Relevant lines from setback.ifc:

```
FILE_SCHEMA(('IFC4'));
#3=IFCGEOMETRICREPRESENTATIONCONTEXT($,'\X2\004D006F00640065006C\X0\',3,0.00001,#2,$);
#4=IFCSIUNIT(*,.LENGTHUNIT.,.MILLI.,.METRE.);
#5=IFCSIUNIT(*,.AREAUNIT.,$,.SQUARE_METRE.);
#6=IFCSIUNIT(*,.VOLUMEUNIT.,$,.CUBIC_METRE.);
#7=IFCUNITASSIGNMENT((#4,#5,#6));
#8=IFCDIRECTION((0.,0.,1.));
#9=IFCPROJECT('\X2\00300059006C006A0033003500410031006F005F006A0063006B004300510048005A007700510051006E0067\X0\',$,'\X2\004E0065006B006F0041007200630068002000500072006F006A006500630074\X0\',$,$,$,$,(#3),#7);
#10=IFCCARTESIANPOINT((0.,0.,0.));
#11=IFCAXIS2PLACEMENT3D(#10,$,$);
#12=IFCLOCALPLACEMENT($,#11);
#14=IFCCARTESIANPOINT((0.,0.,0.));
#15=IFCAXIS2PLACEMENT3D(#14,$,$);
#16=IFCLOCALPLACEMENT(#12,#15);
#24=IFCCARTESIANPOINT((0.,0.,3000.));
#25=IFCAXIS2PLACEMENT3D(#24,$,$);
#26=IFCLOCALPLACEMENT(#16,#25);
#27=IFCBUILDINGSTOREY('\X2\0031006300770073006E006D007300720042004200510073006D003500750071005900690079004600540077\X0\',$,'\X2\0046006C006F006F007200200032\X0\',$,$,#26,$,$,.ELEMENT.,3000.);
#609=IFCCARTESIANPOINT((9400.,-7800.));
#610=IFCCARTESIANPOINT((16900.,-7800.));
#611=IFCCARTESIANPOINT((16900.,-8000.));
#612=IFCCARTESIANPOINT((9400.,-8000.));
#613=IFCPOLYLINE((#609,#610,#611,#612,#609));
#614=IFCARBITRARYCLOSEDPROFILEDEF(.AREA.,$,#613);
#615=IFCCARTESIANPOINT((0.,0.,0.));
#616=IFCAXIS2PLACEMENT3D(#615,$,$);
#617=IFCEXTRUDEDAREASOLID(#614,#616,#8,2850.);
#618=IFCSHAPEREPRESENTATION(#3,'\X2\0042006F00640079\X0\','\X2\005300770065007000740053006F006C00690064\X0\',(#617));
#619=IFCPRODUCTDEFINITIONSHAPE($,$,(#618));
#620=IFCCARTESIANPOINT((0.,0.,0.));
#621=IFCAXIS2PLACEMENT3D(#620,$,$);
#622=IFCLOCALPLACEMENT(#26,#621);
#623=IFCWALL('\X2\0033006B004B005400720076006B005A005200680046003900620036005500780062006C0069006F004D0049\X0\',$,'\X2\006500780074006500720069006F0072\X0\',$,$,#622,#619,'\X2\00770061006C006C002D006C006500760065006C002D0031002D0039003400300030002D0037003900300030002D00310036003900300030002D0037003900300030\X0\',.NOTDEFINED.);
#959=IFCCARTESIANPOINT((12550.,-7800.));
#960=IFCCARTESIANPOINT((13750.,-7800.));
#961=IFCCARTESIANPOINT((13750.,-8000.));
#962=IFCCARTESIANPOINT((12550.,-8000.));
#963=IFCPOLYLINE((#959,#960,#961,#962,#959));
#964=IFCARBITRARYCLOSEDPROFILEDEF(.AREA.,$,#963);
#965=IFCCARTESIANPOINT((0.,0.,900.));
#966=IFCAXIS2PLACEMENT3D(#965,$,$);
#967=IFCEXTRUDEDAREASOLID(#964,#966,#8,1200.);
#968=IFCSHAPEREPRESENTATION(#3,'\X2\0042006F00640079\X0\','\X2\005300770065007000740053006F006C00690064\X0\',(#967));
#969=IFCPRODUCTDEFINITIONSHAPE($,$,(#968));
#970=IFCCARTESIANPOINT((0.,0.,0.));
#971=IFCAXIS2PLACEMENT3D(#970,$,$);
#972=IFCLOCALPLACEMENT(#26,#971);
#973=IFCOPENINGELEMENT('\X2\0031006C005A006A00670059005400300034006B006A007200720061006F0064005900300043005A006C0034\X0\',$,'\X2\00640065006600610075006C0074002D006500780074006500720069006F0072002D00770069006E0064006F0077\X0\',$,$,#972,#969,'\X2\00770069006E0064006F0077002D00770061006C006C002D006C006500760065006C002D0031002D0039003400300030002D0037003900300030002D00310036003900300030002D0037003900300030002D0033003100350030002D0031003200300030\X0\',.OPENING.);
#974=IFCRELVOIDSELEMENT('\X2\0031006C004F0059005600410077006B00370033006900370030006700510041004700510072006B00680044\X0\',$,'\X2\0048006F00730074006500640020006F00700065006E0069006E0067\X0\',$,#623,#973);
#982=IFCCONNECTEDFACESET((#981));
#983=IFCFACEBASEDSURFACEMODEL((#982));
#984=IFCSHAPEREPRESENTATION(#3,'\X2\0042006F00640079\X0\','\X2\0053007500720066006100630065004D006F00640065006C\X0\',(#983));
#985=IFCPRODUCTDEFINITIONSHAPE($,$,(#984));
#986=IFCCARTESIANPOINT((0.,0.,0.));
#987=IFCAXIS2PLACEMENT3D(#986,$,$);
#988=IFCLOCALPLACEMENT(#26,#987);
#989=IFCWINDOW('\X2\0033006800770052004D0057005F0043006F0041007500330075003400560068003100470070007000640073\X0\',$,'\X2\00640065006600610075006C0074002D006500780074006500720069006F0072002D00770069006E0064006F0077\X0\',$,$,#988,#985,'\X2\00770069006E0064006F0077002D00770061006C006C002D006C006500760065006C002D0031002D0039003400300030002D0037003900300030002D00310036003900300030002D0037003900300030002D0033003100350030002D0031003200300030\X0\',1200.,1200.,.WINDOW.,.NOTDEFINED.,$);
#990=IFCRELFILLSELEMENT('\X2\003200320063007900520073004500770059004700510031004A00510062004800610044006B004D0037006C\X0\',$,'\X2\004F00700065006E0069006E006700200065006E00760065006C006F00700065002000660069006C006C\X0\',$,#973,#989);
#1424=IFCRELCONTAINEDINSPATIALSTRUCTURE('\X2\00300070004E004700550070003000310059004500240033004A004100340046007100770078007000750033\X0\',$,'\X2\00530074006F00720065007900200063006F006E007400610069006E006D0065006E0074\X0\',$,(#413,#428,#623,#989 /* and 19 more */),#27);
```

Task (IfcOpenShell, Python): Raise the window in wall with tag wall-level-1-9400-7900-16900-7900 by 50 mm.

```python
import numpy as np
import ifcopenshell
import ifcopenshell.api.geometry
import ifcopenshell.util.placement
import ifcopenshell.util.unit

model = ifcopenshell.open("setback.ifc")
unit_scale = ifcopenshell.util.unit.calculate_unit_scale(model)

window = model.by_id(989)
opening = window.FillsVoids[0].RelatingOpeningElement
dz = 0.05 / unit_scale

shift = np.array([0.0, 0.0, dz])
# The window is not placed relative to its opening, so move both.
for product in (opening, window):
    matrix = ifcopenshell.util.placement.get_local_placement(product.ObjectPlacement)
    matrix[:3, 3] += shift
    ifcopenshell.api.geometry.edit_object_placement(model, product=product, matrix=matrix, is_si=False)

print(f"moved by {dz * unit_scale:+.3f} m")

model.write("setback-out.ifc")
```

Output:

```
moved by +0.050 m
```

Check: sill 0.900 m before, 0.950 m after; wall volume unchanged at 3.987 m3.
